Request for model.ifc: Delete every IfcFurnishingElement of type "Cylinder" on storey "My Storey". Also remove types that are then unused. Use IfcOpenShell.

First a look at what the model holds.

```python
import ifcopenshell
import ifcopenshell.util.element

model = ifcopenshell.open("model.ifc")
print(model.schema)
storey = next(s for s in model.by_type("IfcBuildingStorey") if s.Name == "My Storey")
furniture = [e for e in ifcopenshell.util.element.get_decomposition(storey) if e.is_a("IfcFurnishingElement")]
seen = {}
for e in furniture:
    element_type = ifcopenshell.util.element.get_type(e)
    name = element_type.Name if element_type not in (None, e) else None
    seen[name] = seen.get(name, 0) + 1
for name, count in sorted(seen.items(), key=str):
    print(count, "x", name)
```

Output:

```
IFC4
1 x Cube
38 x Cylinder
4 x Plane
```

```python
import ifcopenshell
import ifcopenshell.api.root
import ifcopenshell.util.element

model = ifcopenshell.open("model.ifc")

storey = next(s for s in model.by_type("IfcBuildingStorey") if s.Name == "My Storey")
furniture = [e for e in ifcopenshell.util.element.get_decomposition(storey) if e.is_a("IfcFurnishingElement")]
targets = [e for e in furniture if (t := ifcopenshell.util.element.get_type(e)) not in (None, e) and t.Name == "Cylinder"]
types = {ifcopenshell.util.element.get_type(e) for e in targets} - {None, *targets}

for e in targets:
    ifcopenshell.api.root.remove_product(model, product=e)
print(len(targets), "removed")

unused = [t for t in types if not ifcopenshell.util.element.get_types(t)]
for t in unused:
    ifcopenshell.api.root.remove_product(model, product=t)
print(len(unused), "unused types removed")

model.write("model_v2.ifc")
```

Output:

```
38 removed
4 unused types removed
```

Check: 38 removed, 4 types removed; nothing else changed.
